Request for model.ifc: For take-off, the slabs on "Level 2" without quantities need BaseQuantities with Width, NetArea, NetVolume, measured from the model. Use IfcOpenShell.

First a look at what the model holds.

```python
import ifcopenshell
import ifcopenshell.util.element
import ifcopenshell.util.unit

model = ifcopenshell.open("model.ifc")
print(model.schema)
for unit_type in ("LENGTHUNIT", "AREAUNIT", "VOLUMEUNIT"):
    print(unit_type, ifcopenshell.util.unit.calculate_unit_scale(model, unit_type))
storey = next(s for s in model.by_type("IfcBuildingStorey") if s.Name == "Level 2")
slabs = [e for e in ifcopenshell.util.element.get_decomposition(storey) if e.is_a("IfcSlab")]
for e in sorted(slabs, key=lambda e: e.id()):
    print(e.id(), e.is_a(), e.Name, list(ifcopenshell.util.element.get_psets(e, qtos_only=True)), sep=" | ")
```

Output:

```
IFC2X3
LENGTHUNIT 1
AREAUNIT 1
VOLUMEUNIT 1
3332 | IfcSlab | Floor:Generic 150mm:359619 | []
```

```python
import ifcopenshell
import ifcopenshell.api.pset
import ifcopenshell.geom
import ifcopenshell.util.element
import ifcopenshell.util.shape
import ifcopenshell.util.unit

model = ifcopenshell.open("model.ifc")
unit_scale = ifcopenshell.util.unit.calculate_unit_scale(model)
area_scale = ifcopenshell.util.unit.calculate_unit_scale(model, "AREAUNIT")
volume_scale = ifcopenshell.util.unit.calculate_unit_scale(model, "VOLUMEUNIT")
settings = ifcopenshell.geom.settings()

storey = next(s for s in model.by_type("IfcBuildingStorey") if s.Name == "Level 2")
slabs = [e for e in ifcopenshell.util.element.get_decomposition(storey) if e.is_a("IfcSlab")]

for e in sorted(slabs, key=lambda e: e.id()):
    if ifcopenshell.util.element.get_psets(e, qtos_only=True, should_inherit=False):
        continue
    # Geometry comes back in metres, in the element's own axes.
    shape = ifcopenshell.geom.create_shape(settings, e)
    values = {
        "Width": ifcopenshell.util.shape.get_z(shape.geometry) / unit_scale,
        "NetArea": ifcopenshell.util.shape.get_footprint_area(shape.geometry) / area_scale,
        "NetVolume": ifcopenshell.util.shape.get_volume(shape.geometry) / volume_scale,
    }
    qto = ifcopenshell.api.pset.add_qto(model, product=e, name="BaseQuantities")
    ifcopenshell.api.pset.edit_qto(model, qto=qto, properties=values)
    print(e.id(), {k: round(v, 3) for k, v in values.items()})

model.write("model_v2.ifc")
```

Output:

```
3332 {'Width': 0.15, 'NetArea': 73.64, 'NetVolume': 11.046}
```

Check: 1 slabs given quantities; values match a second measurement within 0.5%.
